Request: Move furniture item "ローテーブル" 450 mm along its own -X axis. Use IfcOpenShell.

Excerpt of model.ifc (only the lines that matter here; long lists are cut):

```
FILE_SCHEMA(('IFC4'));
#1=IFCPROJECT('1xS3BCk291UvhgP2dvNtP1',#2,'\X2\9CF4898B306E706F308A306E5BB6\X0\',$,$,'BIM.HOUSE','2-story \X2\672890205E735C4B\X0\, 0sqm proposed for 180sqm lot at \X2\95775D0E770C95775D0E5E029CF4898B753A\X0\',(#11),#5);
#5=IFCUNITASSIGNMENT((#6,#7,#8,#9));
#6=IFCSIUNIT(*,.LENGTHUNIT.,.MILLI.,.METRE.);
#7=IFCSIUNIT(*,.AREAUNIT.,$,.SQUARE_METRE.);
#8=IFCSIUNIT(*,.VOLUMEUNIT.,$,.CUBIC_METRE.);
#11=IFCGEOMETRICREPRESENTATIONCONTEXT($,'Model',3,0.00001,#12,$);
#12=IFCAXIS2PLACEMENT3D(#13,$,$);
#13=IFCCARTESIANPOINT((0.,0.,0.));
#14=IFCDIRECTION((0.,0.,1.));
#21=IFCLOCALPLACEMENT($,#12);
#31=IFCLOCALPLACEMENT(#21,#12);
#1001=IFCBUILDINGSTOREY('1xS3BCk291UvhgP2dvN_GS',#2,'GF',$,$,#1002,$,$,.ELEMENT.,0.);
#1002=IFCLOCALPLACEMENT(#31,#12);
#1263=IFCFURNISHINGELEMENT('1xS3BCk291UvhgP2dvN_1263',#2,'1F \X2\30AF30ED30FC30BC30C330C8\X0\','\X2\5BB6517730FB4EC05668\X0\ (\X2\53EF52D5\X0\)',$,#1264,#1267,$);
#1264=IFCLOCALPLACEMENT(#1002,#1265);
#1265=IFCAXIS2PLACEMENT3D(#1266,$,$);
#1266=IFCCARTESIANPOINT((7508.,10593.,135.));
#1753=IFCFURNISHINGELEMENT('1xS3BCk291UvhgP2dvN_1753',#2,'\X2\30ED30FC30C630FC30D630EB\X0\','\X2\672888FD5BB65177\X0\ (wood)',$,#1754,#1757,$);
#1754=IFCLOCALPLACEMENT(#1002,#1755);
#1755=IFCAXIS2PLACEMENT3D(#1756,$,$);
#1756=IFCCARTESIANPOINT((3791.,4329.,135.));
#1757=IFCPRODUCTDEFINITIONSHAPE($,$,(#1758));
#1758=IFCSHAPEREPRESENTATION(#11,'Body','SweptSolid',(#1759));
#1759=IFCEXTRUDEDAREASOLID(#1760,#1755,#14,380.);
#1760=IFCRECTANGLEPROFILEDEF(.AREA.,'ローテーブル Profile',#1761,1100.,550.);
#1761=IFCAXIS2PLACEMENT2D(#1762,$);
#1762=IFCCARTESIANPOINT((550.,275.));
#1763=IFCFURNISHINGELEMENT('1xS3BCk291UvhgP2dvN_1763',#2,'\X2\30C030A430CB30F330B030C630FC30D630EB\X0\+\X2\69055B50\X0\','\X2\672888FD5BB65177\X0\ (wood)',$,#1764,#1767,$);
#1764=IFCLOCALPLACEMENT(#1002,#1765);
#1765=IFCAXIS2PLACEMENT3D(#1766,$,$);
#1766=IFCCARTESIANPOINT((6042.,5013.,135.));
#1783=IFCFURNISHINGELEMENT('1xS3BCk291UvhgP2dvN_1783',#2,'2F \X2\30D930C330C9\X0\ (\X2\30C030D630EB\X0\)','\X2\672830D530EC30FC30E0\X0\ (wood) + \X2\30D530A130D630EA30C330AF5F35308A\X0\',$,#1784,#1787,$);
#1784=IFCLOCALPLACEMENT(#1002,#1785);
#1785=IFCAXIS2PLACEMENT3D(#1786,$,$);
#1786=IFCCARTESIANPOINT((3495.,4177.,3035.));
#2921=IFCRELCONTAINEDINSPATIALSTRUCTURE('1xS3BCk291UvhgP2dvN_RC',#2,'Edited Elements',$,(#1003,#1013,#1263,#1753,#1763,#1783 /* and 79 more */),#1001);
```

```python
import ifcopenshell
import ifcopenshell.api.geometry
import ifcopenshell.util.placement
import ifcopenshell.util.unit

model = ifcopenshell.open("model.ifc")
unit_scale = ifcopenshell.util.unit.calculate_unit_scale(model)

item = model.by_guid("1xS3BCk291UvhgP2dvN_1753")
matrix = ifcopenshell.util.placement.get_local_placement(item.ObjectPlacement)
matrix[:3, 3] -= matrix[:3, 0] * 0.45 / unit_scale
ifcopenshell.api.geometry.edit_object_placement(model, product=item, matrix=matrix, is_si=False)

print(ifcopenshell.util.placement.get_local_placement(item.ObjectPlacement).round(3) + 0.0)

model.write("model_edited.ifc")
```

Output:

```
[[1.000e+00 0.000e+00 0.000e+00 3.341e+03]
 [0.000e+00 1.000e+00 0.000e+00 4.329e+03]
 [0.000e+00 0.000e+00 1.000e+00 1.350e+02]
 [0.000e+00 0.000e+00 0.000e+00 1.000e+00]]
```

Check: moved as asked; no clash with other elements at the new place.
